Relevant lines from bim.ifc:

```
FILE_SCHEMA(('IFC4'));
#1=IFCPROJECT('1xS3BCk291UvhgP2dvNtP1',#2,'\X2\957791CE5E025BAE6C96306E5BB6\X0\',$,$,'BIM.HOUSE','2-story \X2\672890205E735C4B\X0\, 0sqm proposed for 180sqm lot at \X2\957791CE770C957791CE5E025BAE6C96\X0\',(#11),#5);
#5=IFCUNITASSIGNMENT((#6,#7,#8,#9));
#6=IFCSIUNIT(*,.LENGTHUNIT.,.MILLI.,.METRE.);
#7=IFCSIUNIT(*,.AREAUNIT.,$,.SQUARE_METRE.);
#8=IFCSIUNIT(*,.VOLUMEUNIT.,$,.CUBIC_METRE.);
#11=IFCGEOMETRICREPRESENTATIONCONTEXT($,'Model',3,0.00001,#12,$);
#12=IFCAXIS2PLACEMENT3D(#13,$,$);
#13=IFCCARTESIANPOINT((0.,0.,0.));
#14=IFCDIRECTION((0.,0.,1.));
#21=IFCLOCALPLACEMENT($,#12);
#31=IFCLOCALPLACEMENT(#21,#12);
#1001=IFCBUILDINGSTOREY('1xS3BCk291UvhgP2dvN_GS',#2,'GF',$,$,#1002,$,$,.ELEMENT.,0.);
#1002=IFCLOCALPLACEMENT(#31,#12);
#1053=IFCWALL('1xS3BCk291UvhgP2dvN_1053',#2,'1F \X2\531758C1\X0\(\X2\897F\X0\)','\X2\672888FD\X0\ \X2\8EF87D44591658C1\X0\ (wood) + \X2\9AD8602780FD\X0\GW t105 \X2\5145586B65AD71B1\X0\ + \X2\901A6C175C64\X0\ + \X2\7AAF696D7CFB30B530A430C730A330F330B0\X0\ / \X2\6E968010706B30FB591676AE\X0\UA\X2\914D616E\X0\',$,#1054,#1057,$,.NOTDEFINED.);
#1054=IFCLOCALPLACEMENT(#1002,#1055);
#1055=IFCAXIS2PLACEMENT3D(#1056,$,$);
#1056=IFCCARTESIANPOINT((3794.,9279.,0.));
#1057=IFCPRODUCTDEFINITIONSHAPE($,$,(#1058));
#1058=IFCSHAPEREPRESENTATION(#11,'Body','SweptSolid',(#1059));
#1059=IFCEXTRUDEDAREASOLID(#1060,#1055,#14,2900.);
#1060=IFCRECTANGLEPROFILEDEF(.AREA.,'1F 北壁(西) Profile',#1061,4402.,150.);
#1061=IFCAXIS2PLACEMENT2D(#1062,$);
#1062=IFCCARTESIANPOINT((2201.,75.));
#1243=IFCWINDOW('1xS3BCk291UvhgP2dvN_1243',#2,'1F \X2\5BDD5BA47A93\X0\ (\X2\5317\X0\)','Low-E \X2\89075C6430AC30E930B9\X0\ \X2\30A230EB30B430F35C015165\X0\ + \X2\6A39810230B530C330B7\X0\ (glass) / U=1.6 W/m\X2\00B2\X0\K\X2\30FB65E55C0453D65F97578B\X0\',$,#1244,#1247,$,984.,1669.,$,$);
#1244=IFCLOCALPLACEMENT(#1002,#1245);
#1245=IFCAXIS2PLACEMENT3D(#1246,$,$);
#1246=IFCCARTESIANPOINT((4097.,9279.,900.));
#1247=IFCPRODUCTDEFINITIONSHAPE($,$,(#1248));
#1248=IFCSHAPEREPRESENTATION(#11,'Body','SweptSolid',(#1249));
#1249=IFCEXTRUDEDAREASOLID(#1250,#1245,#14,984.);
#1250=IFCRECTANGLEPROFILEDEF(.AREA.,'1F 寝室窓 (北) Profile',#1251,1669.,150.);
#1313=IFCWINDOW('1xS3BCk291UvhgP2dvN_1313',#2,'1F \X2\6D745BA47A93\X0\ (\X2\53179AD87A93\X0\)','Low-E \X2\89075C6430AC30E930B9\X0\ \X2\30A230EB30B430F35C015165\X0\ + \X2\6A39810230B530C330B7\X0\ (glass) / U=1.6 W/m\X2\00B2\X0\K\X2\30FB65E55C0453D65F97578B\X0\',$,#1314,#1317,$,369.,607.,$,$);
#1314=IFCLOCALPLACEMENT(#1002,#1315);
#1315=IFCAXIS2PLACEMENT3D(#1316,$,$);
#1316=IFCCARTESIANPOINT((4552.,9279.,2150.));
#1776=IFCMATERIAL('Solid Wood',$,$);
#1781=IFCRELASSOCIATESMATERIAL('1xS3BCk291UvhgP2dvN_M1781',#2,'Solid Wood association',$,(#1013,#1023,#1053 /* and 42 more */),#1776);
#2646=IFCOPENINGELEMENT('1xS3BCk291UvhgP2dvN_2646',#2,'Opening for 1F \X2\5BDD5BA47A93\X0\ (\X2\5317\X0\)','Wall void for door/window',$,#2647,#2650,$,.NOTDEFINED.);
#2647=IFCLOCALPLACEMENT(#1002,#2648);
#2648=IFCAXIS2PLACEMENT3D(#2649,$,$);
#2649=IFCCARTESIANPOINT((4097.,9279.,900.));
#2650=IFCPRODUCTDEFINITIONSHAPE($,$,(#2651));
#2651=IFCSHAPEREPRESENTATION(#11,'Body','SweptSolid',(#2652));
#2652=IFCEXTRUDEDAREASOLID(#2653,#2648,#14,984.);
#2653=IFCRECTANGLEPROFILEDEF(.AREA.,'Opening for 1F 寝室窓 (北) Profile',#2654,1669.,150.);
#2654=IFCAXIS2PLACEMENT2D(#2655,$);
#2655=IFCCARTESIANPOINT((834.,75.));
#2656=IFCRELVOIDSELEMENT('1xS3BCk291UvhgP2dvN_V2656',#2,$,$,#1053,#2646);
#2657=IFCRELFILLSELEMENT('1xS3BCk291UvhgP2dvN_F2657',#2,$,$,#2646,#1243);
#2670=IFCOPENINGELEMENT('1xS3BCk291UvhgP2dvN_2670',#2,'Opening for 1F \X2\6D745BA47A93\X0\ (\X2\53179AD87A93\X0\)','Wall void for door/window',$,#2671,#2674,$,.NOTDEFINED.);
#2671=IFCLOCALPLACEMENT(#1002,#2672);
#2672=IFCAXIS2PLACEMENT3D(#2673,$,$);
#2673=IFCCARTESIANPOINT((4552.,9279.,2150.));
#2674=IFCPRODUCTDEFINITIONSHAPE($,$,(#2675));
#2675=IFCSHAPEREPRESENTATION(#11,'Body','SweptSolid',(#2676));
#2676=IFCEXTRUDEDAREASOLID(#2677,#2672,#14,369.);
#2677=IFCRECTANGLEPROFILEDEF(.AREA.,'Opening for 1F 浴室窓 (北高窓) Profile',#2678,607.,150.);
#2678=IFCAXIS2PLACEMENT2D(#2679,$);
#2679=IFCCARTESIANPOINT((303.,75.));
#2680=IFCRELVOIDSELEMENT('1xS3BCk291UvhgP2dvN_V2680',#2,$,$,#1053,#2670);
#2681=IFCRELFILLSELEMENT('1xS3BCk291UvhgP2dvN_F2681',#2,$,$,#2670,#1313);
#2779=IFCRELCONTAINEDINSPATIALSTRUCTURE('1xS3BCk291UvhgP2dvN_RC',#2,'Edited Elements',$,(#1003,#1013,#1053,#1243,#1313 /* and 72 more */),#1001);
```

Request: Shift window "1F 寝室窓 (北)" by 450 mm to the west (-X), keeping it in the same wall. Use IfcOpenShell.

```python
import ifcopenshell
import ifcopenshell.api.geometry
import ifcopenshell.util.placement

model = ifcopenshell.open("bim.ifc")

window = model.by_id(1243)
opening = window.FillsVoids[0].RelatingOpeningElement
wall = opening.VoidsElements[0].RelatingBuildingElement

wall_matrix = ifcopenshell.util.placement.get_local_placement(wall.ObjectPlacement)
shift = wall_matrix[:3, 0] * -450.0
before = ifcopenshell.util.placement.get_local_placement(window.ObjectPlacement)[:3, 3].copy()

# The window is not placed relative to its opening, so move both.
for product in (opening, window):
    matrix = ifcopenshell.util.placement.get_local_placement(product.ObjectPlacement)
    matrix[:3, 3] += shift
    ifcopenshell.api.geometry.edit_object_placement(model, product=product, matrix=matrix, is_si=False)

after = ifcopenshell.util.placement.get_local_placement(window.ObjectPlacement)[:3, 3]
print("window moved by", (after - before).round(3) + 0.0)

model.write("bim_rev.ifc")
```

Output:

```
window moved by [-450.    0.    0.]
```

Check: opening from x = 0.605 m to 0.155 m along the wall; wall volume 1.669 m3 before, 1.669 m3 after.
